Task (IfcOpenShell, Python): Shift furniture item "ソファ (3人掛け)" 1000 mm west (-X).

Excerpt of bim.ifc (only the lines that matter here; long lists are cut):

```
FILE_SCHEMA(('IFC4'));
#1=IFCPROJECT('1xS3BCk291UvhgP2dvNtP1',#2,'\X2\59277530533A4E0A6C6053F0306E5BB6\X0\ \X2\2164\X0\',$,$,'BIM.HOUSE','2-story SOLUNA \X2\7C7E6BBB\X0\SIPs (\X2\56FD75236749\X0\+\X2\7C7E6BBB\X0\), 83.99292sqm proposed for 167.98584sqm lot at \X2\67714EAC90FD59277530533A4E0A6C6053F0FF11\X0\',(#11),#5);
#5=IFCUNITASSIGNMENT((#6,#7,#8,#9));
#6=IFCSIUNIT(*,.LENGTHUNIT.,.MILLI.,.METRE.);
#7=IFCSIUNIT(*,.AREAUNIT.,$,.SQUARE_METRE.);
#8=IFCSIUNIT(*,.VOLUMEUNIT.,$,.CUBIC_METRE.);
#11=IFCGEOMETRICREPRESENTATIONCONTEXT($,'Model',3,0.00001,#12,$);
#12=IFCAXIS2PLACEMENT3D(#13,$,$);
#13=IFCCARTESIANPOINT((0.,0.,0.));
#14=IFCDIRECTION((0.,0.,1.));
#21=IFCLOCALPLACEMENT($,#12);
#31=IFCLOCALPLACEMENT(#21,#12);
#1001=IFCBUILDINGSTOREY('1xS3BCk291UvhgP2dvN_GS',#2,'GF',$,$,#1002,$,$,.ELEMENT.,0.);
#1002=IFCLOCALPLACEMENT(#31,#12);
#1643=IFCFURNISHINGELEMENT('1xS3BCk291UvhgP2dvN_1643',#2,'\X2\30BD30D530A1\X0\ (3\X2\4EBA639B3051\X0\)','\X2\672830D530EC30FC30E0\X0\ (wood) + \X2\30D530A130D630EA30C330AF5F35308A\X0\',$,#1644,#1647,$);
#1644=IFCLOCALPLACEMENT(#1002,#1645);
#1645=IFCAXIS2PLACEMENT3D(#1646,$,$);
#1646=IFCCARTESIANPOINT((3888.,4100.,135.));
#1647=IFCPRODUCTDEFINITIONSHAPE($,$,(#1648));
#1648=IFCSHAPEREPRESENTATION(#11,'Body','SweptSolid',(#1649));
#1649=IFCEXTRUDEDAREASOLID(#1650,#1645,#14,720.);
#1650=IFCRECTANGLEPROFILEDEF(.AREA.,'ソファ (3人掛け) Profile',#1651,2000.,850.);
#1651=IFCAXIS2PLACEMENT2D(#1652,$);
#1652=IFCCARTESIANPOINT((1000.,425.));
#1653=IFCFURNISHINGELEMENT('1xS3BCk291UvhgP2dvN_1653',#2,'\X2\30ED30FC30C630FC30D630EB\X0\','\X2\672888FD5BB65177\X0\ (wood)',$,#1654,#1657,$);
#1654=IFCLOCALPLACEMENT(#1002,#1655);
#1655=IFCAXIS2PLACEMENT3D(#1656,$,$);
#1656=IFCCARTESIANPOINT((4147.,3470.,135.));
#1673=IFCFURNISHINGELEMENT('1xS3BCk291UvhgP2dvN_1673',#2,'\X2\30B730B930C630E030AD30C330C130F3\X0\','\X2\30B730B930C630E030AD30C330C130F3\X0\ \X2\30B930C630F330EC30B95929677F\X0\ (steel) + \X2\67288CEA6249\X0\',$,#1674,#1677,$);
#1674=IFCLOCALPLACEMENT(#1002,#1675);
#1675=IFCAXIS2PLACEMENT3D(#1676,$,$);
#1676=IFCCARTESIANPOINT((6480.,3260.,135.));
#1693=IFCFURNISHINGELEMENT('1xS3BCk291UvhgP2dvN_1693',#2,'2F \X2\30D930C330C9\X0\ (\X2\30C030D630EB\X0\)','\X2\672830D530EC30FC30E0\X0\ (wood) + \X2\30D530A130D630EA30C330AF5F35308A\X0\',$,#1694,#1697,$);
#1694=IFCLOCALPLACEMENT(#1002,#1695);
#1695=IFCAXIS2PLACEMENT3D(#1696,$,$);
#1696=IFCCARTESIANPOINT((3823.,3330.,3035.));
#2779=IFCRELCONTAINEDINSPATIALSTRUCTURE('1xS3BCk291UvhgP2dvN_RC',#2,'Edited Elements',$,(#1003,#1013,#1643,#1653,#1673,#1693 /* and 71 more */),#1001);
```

```python
import ifcopenshell
import ifcopenshell.api.geometry
import ifcopenshell.util.placement
import ifcopenshell.util.unit

model = ifcopenshell.open("bim.ifc")
unit_scale = ifcopenshell.util.unit.calculate_unit_scale(model)

item = model.by_guid("1xS3BCk291UvhgP2dvN_1643")
matrix = ifcopenshell.util.placement.get_local_placement(item.ObjectPlacement)
matrix[0, 3] -= 1 / unit_scale
ifcopenshell.api.geometry.edit_object_placement(model, product=item, matrix=matrix, is_si=False)

print(ifcopenshell.util.placement.get_local_placement(item.ObjectPlacement).round(3) + 0.0)

model.write("bim_v2.ifc")
```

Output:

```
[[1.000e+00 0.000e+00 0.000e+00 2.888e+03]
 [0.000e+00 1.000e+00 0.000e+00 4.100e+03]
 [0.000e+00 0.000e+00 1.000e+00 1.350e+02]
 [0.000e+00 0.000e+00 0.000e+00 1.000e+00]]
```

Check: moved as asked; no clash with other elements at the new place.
